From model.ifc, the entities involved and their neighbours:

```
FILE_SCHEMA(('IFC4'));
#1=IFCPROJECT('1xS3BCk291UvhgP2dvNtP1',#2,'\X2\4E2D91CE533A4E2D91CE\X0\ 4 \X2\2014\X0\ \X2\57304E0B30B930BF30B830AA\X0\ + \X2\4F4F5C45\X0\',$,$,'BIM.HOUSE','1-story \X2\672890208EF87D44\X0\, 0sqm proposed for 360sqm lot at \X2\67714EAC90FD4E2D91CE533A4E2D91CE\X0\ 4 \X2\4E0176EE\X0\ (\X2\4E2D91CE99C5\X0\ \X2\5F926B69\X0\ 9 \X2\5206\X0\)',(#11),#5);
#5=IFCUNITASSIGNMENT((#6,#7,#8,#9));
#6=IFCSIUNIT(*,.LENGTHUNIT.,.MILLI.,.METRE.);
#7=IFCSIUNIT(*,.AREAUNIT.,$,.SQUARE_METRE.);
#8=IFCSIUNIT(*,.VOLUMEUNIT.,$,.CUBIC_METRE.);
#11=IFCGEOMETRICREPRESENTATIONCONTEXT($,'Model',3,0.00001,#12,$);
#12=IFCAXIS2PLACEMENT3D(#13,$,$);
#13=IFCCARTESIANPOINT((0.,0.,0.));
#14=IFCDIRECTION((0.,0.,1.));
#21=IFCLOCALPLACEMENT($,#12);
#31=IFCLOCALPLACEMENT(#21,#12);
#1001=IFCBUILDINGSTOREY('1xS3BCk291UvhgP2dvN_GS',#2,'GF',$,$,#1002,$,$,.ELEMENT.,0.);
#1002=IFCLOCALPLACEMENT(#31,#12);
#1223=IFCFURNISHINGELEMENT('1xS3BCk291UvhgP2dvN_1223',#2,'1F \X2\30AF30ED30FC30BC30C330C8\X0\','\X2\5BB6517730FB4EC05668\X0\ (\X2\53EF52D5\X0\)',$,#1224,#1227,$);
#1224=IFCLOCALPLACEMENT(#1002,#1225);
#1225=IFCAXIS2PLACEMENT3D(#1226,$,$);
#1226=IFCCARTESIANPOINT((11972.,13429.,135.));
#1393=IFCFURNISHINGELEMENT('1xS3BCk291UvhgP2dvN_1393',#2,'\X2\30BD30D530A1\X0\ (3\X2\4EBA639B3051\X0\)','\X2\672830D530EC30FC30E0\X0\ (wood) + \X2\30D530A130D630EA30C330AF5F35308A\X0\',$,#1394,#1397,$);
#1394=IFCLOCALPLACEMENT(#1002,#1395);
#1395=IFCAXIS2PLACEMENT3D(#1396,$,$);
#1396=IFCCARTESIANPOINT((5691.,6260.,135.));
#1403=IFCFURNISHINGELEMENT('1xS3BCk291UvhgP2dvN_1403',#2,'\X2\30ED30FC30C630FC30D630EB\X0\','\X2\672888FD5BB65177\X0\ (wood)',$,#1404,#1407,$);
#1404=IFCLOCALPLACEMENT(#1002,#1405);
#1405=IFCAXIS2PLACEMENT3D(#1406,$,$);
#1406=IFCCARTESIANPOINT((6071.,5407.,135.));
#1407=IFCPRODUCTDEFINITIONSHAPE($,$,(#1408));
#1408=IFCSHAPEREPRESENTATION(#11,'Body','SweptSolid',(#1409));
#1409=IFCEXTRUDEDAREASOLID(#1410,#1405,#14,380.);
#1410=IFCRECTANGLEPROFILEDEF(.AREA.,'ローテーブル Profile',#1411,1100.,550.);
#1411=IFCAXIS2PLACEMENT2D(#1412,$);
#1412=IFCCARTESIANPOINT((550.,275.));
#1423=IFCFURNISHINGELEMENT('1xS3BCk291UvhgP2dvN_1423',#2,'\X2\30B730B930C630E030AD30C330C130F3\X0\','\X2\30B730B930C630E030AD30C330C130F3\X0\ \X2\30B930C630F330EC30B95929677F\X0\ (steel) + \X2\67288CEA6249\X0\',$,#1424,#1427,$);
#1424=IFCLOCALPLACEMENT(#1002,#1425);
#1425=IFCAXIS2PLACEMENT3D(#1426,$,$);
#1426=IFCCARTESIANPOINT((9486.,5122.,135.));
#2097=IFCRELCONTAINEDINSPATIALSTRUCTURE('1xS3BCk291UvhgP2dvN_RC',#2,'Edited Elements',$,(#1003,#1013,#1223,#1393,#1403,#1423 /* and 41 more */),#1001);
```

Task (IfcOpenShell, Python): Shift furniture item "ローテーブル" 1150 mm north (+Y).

```python
import ifcopenshell
import ifcopenshell.api.geometry
import ifcopenshell.util.placement
import ifcopenshell.util.unit

model = ifcopenshell.open("model.ifc")
unit_scale = ifcopenshell.util.unit.calculate_unit_scale(model)

item = model.by_guid("1xS3BCk291UvhgP2dvN_1403")
matrix = ifcopenshell.util.placement.get_local_placement(item.ObjectPlacement)
matrix[1, 3] += 1.15 / unit_scale
ifcopenshell.api.geometry.edit_object_placement(model, product=item, matrix=matrix, is_si=False)

print(ifcopenshell.util.placement.get_local_placement(item.ObjectPlacement).round(3) + 0.0)

model.write("model_rev.ifc")
```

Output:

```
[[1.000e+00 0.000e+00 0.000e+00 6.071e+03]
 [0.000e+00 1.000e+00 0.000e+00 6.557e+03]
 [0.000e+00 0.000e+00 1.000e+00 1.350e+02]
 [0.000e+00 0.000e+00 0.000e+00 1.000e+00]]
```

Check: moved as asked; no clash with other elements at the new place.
